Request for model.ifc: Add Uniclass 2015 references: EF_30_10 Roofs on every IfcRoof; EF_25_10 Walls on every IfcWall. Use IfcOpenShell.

First a look at what the model holds.

```python
import ifcopenshell

model = ifcopenshell.open("model.ifc")
print(model.schema)
print("classifications:", [c.Name for c in model.by_type("IfcClassification")])
for ifc_class in ("IfcDoor", "IfcRoof", "IfcStair", "IfcWall", "IfcWindow"):
    print(ifc_class, len(model.by_type(ifc_class)))
```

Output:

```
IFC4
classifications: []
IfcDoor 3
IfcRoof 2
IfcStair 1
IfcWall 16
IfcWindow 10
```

```python
import ifcopenshell
import ifcopenshell.api.classification

model = ifcopenshell.open("model.ifc")

system = ifcopenshell.api.classification.add_classification(model, classification="Uniclass 2015")

codes = {
    "IfcRoof": ("EF_30_10", "Roofs"),
    "IfcWall": ("EF_25_10", "Walls"),
}
for ifc_class, (code, name) in codes.items():
    products = model.by_type(ifc_class)
    ifcopenshell.api.classification.add_reference(
        model, products=products, classification=system, identification=code, name=name
    )
    print(code, len(products))

model.write("model_v2.ifc")
```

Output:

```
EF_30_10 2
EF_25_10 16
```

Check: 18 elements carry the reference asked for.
